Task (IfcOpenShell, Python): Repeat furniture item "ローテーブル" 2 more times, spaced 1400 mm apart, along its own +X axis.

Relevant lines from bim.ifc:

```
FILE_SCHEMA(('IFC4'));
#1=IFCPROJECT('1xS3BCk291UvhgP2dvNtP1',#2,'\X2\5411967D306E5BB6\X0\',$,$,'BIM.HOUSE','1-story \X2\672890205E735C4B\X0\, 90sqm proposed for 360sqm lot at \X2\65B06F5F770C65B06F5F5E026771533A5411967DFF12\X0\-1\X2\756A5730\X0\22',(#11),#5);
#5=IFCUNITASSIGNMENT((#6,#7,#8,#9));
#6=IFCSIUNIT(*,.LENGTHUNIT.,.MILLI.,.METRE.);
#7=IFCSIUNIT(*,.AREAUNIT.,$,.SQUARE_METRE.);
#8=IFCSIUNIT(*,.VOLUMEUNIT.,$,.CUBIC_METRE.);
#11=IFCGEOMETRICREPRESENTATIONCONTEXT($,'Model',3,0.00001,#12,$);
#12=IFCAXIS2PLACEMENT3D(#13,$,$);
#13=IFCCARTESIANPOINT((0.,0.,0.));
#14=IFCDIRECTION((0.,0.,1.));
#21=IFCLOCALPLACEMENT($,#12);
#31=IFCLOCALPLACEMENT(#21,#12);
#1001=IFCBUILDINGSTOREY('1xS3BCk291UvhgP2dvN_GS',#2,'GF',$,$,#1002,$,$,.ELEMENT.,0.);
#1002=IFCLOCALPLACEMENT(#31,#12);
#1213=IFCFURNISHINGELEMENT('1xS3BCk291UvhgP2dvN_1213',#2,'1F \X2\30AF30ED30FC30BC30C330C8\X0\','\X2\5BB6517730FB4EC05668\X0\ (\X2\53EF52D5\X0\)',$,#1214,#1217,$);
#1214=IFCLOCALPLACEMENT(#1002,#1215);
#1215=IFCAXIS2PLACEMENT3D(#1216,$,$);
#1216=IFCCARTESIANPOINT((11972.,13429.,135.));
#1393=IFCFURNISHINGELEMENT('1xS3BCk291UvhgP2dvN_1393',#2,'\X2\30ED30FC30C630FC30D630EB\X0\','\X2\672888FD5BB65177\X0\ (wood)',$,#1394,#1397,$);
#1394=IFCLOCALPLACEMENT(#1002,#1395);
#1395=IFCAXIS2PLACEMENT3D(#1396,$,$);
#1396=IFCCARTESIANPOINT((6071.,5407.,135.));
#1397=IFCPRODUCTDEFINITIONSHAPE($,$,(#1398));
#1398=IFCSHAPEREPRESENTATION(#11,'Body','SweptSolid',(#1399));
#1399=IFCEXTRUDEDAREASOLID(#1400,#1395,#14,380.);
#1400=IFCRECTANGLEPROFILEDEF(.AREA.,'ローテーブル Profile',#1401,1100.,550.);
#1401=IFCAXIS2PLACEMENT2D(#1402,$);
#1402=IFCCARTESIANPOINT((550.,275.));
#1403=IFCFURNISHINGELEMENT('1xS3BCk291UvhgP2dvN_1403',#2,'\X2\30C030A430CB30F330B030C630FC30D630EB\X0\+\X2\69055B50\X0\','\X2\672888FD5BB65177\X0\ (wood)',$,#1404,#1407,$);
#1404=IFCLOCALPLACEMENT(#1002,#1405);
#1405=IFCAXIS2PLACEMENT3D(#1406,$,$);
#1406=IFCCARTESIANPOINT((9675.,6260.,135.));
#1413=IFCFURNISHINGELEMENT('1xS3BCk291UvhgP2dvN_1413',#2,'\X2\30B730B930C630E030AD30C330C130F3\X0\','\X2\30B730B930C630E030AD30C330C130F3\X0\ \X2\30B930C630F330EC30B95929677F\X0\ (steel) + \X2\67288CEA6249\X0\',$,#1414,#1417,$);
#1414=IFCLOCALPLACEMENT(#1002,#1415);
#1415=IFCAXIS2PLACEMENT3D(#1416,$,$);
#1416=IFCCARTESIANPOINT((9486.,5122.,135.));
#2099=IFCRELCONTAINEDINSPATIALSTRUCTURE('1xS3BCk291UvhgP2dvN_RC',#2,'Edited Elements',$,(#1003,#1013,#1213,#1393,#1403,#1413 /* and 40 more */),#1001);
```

```python
import ifcopenshell
import ifcopenshell.api.geometry
import ifcopenshell.api.root
import ifcopenshell.util.element
import ifcopenshell.util.placement
import ifcopenshell.util.unit

model = ifcopenshell.open("bim.ifc")
unit_scale = ifcopenshell.util.unit.calculate_unit_scale(model)


def reuse_history(source, copy):
    """copy_class also copies each property set's owner history, people and application; keep the originals."""
    for rel in copy.IsDefinedBy:
        if rel.is_a("IfcRelDefinesByProperties") and (history := rel.RelatingPropertyDefinition.OwnerHistory):
            rel.RelatingPropertyDefinition.OwnerHistory = source.OwnerHistory
            ifcopenshell.util.element.remove_deep2(model, history)


source = model.by_guid("1xS3BCk291UvhgP2dvN_1393")
base = ifcopenshell.util.placement.get_local_placement(source.ObjectPlacement)
step = base[:3, 0] * 1.4 / unit_scale

for i in range(1, 3):
    copy = ifcopenshell.api.root.copy_class(model, product=source)
    copy.Representation = ifcopenshell.util.element.copy_deep(
        model, source.Representation, exclude=["IfcGeometricRepresentationContext", "IfcRepresentationMap"]
    )
    reuse_history(source, copy)
    matrix = base.copy()
    matrix[:3, 3] += i * step
    print("added at", matrix[:3, 3].round(3) + 0.0)
    ifcopenshell.api.geometry.edit_object_placement(model, product=copy, matrix=matrix, is_si=False)

model.write("bim_updated.ifc")
```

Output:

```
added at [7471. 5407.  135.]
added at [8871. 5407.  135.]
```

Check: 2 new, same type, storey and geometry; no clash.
